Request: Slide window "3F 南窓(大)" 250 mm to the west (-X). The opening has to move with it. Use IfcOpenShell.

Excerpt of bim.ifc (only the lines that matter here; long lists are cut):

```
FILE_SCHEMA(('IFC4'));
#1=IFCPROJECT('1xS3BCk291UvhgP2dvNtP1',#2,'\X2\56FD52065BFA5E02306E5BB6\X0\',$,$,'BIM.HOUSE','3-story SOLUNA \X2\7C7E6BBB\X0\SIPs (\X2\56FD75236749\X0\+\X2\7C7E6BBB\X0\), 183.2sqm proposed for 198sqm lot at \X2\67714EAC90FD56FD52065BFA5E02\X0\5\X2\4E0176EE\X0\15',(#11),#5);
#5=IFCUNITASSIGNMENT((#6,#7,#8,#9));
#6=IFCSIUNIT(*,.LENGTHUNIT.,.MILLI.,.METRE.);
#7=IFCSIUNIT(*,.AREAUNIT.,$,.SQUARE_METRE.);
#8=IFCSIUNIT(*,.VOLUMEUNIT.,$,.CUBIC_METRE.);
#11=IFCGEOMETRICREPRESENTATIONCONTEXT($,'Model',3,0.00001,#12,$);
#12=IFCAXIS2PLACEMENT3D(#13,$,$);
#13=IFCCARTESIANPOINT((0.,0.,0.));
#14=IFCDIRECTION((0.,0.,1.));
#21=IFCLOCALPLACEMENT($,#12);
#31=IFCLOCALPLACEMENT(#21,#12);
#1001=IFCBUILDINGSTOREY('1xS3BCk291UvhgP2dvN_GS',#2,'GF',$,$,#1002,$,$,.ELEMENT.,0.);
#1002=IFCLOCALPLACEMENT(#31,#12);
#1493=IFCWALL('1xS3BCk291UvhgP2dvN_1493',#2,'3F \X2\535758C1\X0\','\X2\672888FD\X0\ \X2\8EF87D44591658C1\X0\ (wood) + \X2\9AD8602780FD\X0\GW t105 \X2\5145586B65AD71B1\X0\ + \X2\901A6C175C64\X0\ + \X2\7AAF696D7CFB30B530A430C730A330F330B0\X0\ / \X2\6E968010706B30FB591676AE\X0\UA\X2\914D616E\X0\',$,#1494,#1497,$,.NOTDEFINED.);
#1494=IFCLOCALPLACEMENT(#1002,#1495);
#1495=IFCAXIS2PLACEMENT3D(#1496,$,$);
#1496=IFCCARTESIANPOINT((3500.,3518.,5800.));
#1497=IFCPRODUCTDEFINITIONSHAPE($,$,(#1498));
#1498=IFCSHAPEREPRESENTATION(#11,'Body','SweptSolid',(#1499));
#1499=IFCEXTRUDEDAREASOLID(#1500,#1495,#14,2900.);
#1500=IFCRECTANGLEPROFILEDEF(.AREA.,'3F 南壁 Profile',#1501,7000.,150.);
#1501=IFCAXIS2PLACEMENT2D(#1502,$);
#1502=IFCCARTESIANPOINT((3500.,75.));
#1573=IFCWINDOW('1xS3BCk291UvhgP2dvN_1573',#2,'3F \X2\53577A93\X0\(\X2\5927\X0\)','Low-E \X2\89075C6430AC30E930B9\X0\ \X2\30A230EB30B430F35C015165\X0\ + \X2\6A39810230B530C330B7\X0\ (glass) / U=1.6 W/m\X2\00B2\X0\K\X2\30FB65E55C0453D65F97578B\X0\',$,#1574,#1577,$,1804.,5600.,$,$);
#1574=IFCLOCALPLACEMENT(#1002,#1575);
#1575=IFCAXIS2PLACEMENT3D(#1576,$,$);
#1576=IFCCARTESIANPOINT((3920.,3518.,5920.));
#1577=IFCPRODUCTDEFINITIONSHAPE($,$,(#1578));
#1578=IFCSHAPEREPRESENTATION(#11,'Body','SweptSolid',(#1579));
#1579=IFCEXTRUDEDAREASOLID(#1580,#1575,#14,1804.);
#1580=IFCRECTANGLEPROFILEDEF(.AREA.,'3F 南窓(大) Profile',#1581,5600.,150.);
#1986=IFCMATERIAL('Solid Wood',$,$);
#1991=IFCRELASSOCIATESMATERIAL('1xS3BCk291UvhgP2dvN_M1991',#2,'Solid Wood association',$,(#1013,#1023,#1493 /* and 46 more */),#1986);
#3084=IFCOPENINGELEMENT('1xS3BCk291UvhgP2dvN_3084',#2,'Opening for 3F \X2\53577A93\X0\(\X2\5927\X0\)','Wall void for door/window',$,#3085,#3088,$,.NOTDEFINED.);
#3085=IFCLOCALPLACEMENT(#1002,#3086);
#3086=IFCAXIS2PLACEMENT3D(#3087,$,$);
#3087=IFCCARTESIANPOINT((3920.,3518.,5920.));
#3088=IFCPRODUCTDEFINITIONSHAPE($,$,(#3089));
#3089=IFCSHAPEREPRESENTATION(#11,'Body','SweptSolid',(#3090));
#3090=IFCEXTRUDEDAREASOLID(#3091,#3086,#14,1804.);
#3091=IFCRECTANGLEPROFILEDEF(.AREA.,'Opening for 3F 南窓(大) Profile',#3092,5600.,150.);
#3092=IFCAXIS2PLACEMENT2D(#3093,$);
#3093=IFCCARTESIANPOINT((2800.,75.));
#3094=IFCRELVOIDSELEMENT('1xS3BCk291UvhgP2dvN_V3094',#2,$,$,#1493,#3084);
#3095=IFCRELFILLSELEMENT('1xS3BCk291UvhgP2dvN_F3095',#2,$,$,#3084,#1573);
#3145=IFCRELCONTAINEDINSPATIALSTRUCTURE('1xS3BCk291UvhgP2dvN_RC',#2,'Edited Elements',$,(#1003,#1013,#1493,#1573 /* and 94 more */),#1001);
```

```python
import ifcopenshell
import ifcopenshell.api.geometry
import ifcopenshell.util.placement
import ifcopenshell.util.unit

model = ifcopenshell.open("bim.ifc")
unit_scale = ifcopenshell.util.unit.calculate_unit_scale(model)

window = model.by_guid("1xS3BCk291UvhgP2dvN_1573")
opening = window.FillsVoids[0].RelatingOpeningElement
wall = opening.VoidsElements[0].RelatingBuildingElement

wall_matrix = ifcopenshell.util.placement.get_local_placement(wall.ObjectPlacement)
shift = wall_matrix[:3, 0] * -0.25 / unit_scale
before = ifcopenshell.util.placement.get_local_placement(window.ObjectPlacement)[:3, 3].copy()

# The window is not placed relative to its opening, so move both.
for product in (opening, window):
    matrix = ifcopenshell.util.placement.get_local_placement(product.ObjectPlacement)
    matrix[:3, 3] += shift
    ifcopenshell.api.geometry.edit_object_placement(model, product=product, matrix=matrix, is_si=False)

after = ifcopenshell.util.placement.get_local_placement(window.ObjectPlacement)[:3, 3]
print("window moved by", (after - before).round(3) + 0.0)

model.write("bim_v2.ifc")
```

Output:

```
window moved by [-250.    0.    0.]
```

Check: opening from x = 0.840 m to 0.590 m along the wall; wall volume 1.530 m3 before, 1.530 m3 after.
